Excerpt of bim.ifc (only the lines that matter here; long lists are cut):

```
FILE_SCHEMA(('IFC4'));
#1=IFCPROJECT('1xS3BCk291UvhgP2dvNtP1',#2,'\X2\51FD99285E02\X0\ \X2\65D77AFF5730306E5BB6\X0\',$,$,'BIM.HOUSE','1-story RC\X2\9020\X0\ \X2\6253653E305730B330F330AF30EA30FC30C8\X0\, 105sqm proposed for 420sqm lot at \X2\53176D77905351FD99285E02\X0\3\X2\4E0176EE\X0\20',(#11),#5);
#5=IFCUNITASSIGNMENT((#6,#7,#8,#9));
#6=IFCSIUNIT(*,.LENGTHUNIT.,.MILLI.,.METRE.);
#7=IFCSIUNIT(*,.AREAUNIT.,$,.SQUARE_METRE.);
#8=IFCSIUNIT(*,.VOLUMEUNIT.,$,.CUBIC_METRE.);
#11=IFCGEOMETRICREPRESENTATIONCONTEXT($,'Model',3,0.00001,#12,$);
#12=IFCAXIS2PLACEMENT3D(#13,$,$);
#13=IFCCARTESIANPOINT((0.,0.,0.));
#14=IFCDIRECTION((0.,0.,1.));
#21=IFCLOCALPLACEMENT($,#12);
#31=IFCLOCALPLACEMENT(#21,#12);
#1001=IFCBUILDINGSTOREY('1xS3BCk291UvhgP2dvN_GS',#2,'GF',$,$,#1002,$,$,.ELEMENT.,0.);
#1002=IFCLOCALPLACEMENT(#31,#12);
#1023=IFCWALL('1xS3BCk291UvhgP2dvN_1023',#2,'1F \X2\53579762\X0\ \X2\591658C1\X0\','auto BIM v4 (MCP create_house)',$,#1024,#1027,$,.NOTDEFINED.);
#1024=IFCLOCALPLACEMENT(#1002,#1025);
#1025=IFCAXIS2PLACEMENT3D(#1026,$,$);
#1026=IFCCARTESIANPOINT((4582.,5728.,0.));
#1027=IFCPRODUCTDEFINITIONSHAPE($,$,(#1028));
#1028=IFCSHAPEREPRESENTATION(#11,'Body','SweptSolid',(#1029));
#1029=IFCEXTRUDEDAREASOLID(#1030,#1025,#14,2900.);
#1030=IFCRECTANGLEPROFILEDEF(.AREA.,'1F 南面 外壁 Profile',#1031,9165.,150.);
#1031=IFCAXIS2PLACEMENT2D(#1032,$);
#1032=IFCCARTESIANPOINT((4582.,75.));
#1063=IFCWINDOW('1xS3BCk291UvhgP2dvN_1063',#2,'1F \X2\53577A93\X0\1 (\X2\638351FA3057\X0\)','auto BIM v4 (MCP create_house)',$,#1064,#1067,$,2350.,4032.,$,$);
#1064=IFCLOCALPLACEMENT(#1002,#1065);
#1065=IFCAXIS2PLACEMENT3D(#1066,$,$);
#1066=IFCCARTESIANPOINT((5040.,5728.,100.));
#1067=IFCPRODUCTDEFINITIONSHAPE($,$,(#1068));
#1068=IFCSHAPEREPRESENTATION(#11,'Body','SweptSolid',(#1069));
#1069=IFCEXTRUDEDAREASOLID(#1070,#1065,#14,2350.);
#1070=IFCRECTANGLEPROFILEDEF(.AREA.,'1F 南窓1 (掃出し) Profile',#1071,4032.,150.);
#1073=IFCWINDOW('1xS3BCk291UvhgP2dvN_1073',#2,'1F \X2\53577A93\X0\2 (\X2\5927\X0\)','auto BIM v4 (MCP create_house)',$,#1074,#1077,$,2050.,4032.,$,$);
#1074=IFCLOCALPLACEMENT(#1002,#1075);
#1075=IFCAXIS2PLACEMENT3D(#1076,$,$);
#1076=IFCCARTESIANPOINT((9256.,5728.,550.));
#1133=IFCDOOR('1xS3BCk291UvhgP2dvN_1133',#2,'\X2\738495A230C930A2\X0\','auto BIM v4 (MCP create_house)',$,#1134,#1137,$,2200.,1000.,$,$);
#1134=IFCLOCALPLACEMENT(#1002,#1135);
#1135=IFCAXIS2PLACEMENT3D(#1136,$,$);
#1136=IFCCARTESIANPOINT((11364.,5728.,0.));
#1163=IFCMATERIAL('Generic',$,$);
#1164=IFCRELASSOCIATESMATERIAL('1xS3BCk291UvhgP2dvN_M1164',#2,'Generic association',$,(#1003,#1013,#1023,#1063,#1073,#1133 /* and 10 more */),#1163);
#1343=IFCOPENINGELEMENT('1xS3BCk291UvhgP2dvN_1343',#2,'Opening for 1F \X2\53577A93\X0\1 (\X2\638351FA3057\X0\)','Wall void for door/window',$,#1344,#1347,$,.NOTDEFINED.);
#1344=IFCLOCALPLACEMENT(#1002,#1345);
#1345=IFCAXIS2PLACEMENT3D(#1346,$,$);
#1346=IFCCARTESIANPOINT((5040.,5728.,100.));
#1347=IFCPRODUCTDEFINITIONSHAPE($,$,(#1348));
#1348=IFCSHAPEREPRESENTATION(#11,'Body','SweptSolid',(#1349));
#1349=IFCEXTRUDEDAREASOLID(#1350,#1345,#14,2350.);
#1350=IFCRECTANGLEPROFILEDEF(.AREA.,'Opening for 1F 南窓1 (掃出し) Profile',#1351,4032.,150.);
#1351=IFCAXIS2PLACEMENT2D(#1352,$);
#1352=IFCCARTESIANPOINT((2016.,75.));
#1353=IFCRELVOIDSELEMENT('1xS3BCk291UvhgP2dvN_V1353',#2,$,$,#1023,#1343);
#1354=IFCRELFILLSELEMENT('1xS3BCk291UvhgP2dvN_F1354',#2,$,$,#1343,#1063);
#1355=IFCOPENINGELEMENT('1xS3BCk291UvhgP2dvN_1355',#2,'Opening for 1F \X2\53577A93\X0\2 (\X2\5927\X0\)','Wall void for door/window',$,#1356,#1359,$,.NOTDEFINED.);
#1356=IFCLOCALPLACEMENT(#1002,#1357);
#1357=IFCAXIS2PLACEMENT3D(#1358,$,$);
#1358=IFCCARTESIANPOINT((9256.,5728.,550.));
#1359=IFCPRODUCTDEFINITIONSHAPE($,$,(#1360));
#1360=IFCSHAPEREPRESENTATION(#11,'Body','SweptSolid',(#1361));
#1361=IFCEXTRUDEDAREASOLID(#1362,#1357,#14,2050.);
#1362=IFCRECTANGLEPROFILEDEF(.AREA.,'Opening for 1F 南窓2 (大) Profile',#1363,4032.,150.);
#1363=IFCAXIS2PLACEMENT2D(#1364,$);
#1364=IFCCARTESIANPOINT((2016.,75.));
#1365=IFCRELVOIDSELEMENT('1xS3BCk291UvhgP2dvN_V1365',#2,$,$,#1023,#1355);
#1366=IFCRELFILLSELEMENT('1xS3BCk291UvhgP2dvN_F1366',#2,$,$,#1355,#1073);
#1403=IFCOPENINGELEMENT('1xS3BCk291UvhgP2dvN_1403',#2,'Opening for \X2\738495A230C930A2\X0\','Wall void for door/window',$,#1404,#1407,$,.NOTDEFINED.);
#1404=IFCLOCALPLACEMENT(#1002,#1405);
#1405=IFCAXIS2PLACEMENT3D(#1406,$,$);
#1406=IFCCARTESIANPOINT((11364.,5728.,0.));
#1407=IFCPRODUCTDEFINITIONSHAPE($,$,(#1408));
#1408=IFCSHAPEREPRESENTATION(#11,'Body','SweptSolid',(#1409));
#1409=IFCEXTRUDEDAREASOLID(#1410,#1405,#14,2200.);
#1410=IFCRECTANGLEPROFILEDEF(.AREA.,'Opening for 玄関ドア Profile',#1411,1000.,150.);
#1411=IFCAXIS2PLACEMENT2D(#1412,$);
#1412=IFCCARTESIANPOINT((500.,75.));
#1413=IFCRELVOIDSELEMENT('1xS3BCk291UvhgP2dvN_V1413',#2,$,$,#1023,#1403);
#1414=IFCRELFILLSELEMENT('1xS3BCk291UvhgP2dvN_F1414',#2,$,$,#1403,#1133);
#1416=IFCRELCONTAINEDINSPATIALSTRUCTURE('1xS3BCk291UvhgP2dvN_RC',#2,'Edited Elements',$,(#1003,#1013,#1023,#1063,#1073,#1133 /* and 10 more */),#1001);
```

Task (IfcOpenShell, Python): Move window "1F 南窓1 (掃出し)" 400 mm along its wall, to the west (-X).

```python
import ifcopenshell
import ifcopenshell.api.geometry
import ifcopenshell.util.placement
import ifcopenshell.util.unit

model = ifcopenshell.open("bim.ifc")
unit_scale = ifcopenshell.util.unit.calculate_unit_scale(model)

window = model.by_guid("1xS3BCk291UvhgP2dvN_1063")
opening = window.FillsVoids[0].RelatingOpeningElement
wall = opening.VoidsElements[0].RelatingBuildingElement

wall_matrix = ifcopenshell.util.placement.get_local_placement(wall.ObjectPlacement)
shift = wall_matrix[:3, 0] * -0.4 / unit_scale
before = ifcopenshell.util.placement.get_local_placement(window.ObjectPlacement)[:3, 3].copy()

# The window is not placed relative to its opening, so move both.
for product in (opening, window):
    matrix = ifcopenshell.util.placement.get_local_placement(product.ObjectPlacement)
    matrix[:3, 3] += shift
    ifcopenshell.api.geometry.edit_object_placement(model, product=product, matrix=matrix, is_si=False)

after = ifcopenshell.util.placement.get_local_placement(window.ObjectPlacement)[:3, 3]
print("window moved by", (after - before).round(3) + 0.0)

model.write("bim-out.ifc")
```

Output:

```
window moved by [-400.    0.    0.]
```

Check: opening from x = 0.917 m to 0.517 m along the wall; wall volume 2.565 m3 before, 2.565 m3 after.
